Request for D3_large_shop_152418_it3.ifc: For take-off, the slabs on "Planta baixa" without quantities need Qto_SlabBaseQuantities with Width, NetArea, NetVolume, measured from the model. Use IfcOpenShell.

First a look at what the model holds.

```python
import ifcopenshell
import ifcopenshell.util.element
import ifcopenshell.util.unit

model = ifcopenshell.open("D3_large_shop_152418_it3.ifc")
print(model.schema)
for unit_type in ("LENGTHUNIT", "AREAUNIT", "VOLUMEUNIT"):
    print(unit_type, ifcopenshell.util.unit.calculate_unit_scale(model, unit_type))
storey = next(s for s in model.by_type("IfcBuildingStorey") if s.Name == "Planta baixa")
slabs = [e for e in ifcopenshell.util.element.get_decomposition(storey) if e.is_a("IfcSlab")]
for e in sorted(slabs, key=lambda e: e.id()):
    print(e.id(), e.is_a(), e.Name, list(ifcopenshell.util.element.get_psets(e, qtos_only=True)), sep=" | ")
```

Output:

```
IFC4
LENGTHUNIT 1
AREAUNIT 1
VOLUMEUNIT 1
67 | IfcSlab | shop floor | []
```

```python
import ifcopenshell
import ifcopenshell.api.pset
import ifcopenshell.geom
import ifcopenshell.util.element
import ifcopenshell.util.shape
import ifcopenshell.util.unit

model = ifcopenshell.open("D3_large_shop_152418_it3.ifc")
unit_scale = ifcopenshell.util.unit.calculate_unit_scale(model)
area_scale = ifcopenshell.util.unit.calculate_unit_scale(model, "AREAUNIT")
volume_scale = ifcopenshell.util.unit.calculate_unit_scale(model, "VOLUMEUNIT")
settings = ifcopenshell.geom.settings()

storey = next(s for s in model.by_type("IfcBuildingStorey") if s.Name == "Planta baixa")
slabs = [e for e in ifcopenshell.util.element.get_decomposition(storey) if e.is_a("IfcSlab")]

for e in sorted(slabs, key=lambda e: e.id()):
    if ifcopenshell.util.element.get_psets(e, qtos_only=True, should_inherit=False):
        continue
    # Geometry comes back in metres, in the element's own axes.
    shape = ifcopenshell.geom.create_shape(settings, e)
    values = {
        "Width": ifcopenshell.util.shape.get_z(shape.geometry) / unit_scale,
        "NetArea": ifcopenshell.util.shape.get_footprint_area(shape.geometry) / area_scale,
        "NetVolume": ifcopenshell.util.shape.get_volume(shape.geometry) / volume_scale,
    }
    qto = ifcopenshell.api.pset.add_qto(model, product=e, name="Qto_SlabBaseQuantities")
    ifcopenshell.api.pset.edit_qto(model, qto=qto, properties=values)
    print(e.id(), {k: round(v, 3) for k, v in values.items()})

model.write("D3_large_shop_152418_it3_v2.ifc")
```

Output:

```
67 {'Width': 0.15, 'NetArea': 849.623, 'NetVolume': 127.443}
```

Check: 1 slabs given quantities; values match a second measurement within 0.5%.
